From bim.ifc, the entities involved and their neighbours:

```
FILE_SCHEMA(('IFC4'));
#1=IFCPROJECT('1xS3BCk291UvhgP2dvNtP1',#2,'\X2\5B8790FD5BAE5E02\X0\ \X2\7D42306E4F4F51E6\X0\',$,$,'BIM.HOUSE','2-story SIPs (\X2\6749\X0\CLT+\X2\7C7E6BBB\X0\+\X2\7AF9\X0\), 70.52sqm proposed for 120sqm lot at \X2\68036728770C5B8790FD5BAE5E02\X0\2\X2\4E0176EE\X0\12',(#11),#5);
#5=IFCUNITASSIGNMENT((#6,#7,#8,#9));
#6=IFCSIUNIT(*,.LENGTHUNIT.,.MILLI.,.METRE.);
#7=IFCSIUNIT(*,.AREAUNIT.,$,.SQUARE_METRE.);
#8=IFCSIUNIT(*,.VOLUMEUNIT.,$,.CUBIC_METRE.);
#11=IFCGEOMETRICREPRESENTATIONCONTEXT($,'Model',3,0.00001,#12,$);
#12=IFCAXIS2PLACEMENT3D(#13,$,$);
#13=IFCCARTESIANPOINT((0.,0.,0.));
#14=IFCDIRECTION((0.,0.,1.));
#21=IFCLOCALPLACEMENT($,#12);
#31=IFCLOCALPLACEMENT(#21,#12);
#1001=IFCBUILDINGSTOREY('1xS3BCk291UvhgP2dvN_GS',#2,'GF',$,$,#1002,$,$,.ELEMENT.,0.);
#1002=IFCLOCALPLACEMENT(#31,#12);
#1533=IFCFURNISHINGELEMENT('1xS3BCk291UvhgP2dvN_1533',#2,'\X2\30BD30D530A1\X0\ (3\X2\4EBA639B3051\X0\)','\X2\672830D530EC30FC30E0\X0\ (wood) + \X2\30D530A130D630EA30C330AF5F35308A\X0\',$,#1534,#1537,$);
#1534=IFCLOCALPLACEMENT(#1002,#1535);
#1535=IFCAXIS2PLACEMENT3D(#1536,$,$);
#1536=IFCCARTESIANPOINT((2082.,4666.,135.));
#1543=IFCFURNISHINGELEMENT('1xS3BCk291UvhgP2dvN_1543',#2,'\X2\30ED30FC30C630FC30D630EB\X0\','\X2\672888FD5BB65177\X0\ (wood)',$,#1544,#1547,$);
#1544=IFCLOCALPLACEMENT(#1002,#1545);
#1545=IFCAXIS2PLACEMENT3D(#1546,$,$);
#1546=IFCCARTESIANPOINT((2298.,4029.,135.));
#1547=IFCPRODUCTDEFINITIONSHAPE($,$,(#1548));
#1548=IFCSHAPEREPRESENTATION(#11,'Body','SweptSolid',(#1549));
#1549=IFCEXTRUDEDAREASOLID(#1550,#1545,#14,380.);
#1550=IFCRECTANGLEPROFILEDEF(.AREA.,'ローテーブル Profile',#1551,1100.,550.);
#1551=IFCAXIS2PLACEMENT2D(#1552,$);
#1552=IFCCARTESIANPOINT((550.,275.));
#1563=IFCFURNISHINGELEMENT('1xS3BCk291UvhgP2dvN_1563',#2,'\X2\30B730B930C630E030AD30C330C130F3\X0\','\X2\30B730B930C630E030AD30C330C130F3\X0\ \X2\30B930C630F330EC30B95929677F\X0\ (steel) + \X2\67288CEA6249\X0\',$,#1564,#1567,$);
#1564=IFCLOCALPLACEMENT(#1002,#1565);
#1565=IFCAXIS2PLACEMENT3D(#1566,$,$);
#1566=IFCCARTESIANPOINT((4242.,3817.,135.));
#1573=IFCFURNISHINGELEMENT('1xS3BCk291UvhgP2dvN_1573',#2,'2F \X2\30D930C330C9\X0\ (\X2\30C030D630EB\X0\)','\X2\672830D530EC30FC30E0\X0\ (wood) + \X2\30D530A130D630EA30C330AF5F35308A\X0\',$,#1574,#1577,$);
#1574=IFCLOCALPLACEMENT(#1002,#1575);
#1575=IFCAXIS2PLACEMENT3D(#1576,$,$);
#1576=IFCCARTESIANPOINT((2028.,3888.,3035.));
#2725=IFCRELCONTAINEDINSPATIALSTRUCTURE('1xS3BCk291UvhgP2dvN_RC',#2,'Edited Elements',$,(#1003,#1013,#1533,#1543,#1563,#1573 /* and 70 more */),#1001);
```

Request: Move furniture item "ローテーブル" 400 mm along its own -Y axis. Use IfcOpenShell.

```python
import ifcopenshell
import ifcopenshell.api.geometry
import ifcopenshell.util.placement
import ifcopenshell.util.unit

model = ifcopenshell.open("bim.ifc")
unit_scale = ifcopenshell.util.unit.calculate_unit_scale(model)

item = model.by_guid("1xS3BCk291UvhgP2dvN_1543")
matrix = ifcopenshell.util.placement.get_local_placement(item.ObjectPlacement)
matrix[:3, 3] -= matrix[:3, 1] * 0.4 / unit_scale
ifcopenshell.api.geometry.edit_object_placement(model, product=item, matrix=matrix, is_si=False)

print(ifcopenshell.util.placement.get_local_placement(item.ObjectPlacement).round(3) + 0.0)

model.write("bim-out.ifc")
```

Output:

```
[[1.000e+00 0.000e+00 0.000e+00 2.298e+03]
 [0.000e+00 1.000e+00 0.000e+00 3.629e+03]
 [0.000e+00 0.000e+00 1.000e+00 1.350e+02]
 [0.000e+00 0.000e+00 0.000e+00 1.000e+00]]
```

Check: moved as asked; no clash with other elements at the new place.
